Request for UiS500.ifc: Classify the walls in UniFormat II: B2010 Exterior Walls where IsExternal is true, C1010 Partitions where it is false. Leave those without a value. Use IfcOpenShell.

First a look at what the model holds.

```python
import ifcopenshell
import ifcopenshell.util.element

model = ifcopenshell.open("UiS500.ifc")
print(model.schema)
print("classifications:", [c.Name for c in model.by_type("IfcClassification")])
values = [ifcopenshell.util.element.get_pset(e, "Pset_WallCommon", "IsExternal") for e in model.by_type("IfcWall")]
for value in (True, False, None):
    print("IsExternal", value, values.count(value))
```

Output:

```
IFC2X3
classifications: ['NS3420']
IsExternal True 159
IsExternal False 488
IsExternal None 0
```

```python
import ifcopenshell
import ifcopenshell.api.classification
import ifcopenshell.util.element

model = ifcopenshell.open("UiS500.ifc")

# IFC2X3 requires Source and Edition and has no link from the project to the system.
system = model.create_entity("IfcClassification", Source="ASTM", Edition="E1557", Name="UniFormat II")

walls = model.by_type("IfcWall")
external = {e: ifcopenshell.util.element.get_pset(e, "Pset_WallCommon", "IsExternal") for e in walls}
for flag, code, name in ((True, "B2010", "Exterior Walls"), (False, "C1010", "Partitions")):
    products = [e for e in walls if external[e] is flag]
    ifcopenshell.api.classification.add_reference(
        model, products=products, classification=system, identification=code, name=name
    )
    print(code, len(products))

model.write("UiS500_updated.ifc")
```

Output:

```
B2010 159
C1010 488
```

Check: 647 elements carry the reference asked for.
